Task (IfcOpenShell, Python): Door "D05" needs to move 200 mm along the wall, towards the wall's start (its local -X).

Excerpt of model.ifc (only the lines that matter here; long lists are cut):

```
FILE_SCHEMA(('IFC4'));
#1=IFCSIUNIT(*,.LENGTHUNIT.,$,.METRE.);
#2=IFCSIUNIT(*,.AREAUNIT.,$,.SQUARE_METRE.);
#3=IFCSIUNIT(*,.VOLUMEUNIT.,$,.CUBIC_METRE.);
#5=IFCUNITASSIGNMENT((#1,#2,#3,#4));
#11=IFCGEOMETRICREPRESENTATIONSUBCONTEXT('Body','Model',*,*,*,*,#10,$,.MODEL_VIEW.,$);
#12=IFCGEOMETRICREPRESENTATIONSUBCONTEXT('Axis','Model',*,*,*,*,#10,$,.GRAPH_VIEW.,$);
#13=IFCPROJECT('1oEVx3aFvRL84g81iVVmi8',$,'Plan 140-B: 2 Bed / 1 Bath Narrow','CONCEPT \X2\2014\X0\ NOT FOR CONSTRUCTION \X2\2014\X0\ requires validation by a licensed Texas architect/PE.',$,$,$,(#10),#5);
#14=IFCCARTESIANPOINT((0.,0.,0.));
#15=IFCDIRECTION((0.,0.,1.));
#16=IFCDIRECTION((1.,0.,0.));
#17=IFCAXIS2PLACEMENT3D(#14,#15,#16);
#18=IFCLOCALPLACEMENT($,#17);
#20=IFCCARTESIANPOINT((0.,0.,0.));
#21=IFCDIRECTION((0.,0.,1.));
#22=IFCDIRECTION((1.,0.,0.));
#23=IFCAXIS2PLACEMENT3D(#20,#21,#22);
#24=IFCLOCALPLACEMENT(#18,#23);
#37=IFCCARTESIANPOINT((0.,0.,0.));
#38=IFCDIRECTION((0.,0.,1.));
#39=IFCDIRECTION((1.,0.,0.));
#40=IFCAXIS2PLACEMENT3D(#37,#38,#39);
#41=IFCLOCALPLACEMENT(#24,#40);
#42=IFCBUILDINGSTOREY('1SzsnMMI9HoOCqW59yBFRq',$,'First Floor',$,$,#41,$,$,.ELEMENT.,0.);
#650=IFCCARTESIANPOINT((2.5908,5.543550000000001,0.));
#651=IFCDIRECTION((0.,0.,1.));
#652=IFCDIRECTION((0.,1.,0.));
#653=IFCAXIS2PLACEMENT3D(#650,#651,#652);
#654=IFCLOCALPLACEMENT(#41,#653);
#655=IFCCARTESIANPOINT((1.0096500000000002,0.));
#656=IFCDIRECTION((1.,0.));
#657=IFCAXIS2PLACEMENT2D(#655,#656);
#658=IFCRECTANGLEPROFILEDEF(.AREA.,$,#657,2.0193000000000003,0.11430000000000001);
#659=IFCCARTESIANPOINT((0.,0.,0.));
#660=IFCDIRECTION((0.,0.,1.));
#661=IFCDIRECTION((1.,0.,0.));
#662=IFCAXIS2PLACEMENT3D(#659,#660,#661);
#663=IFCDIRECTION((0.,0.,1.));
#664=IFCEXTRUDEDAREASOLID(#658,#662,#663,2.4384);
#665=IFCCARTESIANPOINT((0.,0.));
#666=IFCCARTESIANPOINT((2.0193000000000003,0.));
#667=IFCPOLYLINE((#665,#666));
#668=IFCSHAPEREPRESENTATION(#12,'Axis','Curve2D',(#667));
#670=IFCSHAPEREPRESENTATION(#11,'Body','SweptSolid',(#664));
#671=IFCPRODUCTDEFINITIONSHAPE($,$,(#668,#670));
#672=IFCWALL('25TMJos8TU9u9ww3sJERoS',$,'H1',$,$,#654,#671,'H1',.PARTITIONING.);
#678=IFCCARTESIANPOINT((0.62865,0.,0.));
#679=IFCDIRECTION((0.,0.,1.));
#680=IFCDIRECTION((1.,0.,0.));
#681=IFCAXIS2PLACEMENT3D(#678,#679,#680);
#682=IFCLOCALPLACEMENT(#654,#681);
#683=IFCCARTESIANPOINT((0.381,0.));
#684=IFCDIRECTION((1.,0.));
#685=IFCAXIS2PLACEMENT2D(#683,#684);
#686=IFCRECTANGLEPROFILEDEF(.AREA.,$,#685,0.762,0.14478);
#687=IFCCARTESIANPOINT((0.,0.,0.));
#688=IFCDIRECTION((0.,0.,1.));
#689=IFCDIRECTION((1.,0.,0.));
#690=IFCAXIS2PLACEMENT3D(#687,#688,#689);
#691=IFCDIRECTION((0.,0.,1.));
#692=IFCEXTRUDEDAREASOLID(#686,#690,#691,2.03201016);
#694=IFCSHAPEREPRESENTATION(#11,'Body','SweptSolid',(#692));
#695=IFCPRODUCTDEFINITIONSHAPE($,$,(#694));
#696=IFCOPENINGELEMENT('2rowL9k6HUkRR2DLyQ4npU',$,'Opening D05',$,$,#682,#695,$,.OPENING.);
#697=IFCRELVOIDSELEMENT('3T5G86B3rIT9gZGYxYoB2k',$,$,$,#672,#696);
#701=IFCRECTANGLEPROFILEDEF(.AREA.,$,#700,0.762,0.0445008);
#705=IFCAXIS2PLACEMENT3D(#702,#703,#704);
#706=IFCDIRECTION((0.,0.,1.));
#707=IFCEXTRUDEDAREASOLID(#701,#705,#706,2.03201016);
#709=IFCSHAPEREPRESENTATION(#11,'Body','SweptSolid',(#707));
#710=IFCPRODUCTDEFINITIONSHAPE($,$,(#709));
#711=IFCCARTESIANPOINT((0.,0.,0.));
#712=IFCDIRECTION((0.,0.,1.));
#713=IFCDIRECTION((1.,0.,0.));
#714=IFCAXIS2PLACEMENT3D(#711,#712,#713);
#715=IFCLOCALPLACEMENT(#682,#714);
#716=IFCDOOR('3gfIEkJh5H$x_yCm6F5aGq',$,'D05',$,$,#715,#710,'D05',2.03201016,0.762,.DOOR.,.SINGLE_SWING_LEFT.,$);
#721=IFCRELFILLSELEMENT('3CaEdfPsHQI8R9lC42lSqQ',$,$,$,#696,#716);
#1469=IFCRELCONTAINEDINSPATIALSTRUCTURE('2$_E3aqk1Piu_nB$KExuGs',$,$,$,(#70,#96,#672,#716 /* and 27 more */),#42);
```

```python
import ifcopenshell
import ifcopenshell.api.geometry
import ifcopenshell.util.placement

model = ifcopenshell.open("model.ifc")

door = model.by_id(716)
opening = door.FillsVoids[0].RelatingOpeningElement
wall = opening.VoidsElements[0].RelatingBuildingElement

wall_matrix = ifcopenshell.util.placement.get_local_placement(wall.ObjectPlacement)
shift = wall_matrix[:3, 0] * -0.2
before = ifcopenshell.util.placement.get_local_placement(door.ObjectPlacement)[:3, 3].copy()

# The door is placed relative to its opening, so it follows when the opening moves.
matrix = ifcopenshell.util.placement.get_local_placement(opening.ObjectPlacement)
matrix[:3, 3] += shift
ifcopenshell.api.geometry.edit_object_placement(
    model, product=opening, matrix=matrix, is_si=False, should_transform_children=True
)

after = ifcopenshell.util.placement.get_local_placement(door.ObjectPlacement)[:3, 3]
print("door moved by", (after - before).round(3) + 0.0)

model.write("model_updated.ifc")
```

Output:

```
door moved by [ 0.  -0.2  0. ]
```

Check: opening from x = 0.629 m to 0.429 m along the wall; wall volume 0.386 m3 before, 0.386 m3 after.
